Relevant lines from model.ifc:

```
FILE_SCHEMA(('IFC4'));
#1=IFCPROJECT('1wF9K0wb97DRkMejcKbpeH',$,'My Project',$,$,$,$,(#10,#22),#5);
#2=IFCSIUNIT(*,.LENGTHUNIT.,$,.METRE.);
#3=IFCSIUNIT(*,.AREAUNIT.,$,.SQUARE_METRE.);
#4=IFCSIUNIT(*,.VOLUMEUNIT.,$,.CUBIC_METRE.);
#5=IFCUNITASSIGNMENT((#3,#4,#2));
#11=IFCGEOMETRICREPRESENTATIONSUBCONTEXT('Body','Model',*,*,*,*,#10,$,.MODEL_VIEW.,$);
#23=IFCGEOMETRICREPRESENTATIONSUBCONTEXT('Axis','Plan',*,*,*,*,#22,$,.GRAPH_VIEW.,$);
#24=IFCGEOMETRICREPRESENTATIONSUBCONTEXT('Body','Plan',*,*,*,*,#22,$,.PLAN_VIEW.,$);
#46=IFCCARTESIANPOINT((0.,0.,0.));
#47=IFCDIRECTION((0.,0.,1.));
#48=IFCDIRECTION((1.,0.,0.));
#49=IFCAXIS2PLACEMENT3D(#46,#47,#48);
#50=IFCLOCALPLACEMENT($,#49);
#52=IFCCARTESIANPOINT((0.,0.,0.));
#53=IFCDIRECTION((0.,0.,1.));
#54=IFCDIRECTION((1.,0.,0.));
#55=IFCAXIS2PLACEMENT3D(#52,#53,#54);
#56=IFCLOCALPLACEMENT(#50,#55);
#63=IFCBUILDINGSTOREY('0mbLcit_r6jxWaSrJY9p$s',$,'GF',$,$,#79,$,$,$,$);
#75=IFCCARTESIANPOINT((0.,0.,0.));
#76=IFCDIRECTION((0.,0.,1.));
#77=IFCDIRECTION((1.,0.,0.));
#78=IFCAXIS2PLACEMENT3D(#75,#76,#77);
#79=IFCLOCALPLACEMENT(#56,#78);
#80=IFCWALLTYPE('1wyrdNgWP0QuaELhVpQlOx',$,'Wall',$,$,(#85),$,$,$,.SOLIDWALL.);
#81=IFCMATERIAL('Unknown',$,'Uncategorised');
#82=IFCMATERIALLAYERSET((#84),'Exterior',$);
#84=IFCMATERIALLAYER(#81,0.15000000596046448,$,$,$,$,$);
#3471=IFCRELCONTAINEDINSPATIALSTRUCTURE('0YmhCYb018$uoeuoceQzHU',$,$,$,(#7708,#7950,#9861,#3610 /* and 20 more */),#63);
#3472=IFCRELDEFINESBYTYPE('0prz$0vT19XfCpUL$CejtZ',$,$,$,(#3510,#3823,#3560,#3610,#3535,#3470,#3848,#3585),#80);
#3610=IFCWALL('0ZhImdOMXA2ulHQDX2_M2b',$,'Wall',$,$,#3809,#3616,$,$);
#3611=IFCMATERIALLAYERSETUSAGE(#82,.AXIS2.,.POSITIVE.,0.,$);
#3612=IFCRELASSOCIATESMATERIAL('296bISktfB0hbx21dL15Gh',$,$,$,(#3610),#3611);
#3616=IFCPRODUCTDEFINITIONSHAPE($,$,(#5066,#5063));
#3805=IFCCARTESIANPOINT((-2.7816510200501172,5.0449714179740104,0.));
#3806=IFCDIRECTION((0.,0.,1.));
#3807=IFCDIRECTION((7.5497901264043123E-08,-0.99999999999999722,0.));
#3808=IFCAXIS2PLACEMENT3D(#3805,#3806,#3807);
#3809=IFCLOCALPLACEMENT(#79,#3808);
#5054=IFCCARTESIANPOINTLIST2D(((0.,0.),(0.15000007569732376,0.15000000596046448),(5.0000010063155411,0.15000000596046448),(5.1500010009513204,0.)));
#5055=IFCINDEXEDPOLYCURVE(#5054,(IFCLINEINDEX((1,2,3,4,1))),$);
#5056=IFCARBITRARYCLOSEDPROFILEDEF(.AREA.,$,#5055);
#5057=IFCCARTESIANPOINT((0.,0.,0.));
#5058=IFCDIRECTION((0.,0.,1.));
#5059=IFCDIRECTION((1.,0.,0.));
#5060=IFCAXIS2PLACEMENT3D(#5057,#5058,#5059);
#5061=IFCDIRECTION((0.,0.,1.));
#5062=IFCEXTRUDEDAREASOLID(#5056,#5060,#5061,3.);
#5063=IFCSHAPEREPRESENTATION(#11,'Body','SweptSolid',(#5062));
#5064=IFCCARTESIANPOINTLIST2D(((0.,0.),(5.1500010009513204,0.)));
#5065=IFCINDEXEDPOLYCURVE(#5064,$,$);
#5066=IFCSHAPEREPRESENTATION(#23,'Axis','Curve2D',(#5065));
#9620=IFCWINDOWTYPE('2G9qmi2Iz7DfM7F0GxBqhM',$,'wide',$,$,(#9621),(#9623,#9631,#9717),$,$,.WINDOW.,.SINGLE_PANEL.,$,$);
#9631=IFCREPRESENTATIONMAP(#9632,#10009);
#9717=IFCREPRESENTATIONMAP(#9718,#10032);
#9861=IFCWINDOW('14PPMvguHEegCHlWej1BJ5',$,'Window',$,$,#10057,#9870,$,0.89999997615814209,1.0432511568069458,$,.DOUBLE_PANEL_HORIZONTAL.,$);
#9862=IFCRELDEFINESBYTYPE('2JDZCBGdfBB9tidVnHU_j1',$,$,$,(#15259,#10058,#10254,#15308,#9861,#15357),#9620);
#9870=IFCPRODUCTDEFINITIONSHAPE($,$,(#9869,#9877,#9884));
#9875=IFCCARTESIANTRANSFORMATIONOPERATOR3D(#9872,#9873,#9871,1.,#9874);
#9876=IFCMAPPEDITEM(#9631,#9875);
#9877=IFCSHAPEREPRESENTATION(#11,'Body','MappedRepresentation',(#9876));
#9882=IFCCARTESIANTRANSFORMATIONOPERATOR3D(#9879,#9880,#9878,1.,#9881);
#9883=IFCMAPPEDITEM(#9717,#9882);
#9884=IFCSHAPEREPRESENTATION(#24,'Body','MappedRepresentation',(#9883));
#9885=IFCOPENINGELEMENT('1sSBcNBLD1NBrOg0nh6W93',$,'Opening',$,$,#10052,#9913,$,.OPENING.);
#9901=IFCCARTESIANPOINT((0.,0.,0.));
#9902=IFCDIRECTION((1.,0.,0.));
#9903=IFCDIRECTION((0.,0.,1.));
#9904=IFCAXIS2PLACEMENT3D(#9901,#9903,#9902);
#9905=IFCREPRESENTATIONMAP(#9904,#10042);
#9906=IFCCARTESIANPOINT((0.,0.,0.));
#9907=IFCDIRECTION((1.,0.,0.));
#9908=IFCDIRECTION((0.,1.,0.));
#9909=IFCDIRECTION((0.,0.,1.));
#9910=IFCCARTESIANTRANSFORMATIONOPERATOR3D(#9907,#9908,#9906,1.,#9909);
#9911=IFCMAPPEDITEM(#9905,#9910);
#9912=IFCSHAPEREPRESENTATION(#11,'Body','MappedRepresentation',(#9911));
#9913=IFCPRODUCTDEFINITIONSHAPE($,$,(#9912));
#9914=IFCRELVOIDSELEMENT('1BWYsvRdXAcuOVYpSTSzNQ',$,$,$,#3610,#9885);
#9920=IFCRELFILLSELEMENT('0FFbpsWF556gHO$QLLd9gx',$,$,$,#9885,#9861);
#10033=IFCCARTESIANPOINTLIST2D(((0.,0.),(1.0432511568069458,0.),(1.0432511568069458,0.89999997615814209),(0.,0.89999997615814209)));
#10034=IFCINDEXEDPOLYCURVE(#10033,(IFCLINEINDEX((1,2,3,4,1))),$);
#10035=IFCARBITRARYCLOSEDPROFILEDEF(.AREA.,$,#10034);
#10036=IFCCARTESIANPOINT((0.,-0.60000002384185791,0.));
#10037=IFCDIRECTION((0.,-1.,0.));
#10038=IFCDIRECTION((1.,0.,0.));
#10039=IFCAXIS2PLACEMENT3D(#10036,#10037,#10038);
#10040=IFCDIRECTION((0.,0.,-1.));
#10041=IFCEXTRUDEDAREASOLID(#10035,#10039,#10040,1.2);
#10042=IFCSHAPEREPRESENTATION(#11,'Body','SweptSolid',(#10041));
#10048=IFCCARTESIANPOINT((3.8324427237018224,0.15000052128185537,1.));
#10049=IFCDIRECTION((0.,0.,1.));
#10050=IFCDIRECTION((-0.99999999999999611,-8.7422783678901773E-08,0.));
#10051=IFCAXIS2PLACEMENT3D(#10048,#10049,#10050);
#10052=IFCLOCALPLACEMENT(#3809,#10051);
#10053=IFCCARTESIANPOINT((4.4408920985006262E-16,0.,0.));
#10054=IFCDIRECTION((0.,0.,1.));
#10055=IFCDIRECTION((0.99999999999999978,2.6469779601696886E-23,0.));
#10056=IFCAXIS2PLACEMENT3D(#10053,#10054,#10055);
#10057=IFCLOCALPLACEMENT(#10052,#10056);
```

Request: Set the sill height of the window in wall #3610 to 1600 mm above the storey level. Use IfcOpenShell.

```python
import numpy as np
import ifcopenshell
import ifcopenshell.api.geometry
import ifcopenshell.geom
import ifcopenshell.util.element
import ifcopenshell.util.placement
import ifcopenshell.util.shape
import ifcopenshell.util.unit

model = ifcopenshell.open("model.ifc")
unit_scale = ifcopenshell.util.unit.calculate_unit_scale(model)

window = model.by_guid("14PPMvguHEegCHlWej1BJ5")
opening = window.FillsVoids[0].RelatingOpeningElement
storey = ifcopenshell.util.element.get_container(window, ifc_class="IfcBuildingStorey")
level = ifcopenshell.util.placement.get_local_placement(storey.ObjectPlacement)[2, 3]

# The opening's origin need not be at the sill, so measure its lowest point.
shape = ifcopenshell.geom.create_shape(ifcopenshell.geom.settings(), opening)
bottom = ifcopenshell.util.shape.get_shape_bottom_elevation(shape, shape.geometry) / unit_scale
dz = level + 1.6 / unit_scale - bottom

shift = np.array([0.0, 0.0, dz])
# The window is placed relative to its opening, so it follows when the opening moves.
matrix = ifcopenshell.util.placement.get_local_placement(opening.ObjectPlacement)
matrix[:3, 3] += shift
ifcopenshell.api.geometry.edit_object_placement(
    model, product=opening, matrix=matrix, is_si=False, should_transform_children=True
)

print(f"moved by {dz * unit_scale:+.3f} m")

model.write("model_updated.ifc")
```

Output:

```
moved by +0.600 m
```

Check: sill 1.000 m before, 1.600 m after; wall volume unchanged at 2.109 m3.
